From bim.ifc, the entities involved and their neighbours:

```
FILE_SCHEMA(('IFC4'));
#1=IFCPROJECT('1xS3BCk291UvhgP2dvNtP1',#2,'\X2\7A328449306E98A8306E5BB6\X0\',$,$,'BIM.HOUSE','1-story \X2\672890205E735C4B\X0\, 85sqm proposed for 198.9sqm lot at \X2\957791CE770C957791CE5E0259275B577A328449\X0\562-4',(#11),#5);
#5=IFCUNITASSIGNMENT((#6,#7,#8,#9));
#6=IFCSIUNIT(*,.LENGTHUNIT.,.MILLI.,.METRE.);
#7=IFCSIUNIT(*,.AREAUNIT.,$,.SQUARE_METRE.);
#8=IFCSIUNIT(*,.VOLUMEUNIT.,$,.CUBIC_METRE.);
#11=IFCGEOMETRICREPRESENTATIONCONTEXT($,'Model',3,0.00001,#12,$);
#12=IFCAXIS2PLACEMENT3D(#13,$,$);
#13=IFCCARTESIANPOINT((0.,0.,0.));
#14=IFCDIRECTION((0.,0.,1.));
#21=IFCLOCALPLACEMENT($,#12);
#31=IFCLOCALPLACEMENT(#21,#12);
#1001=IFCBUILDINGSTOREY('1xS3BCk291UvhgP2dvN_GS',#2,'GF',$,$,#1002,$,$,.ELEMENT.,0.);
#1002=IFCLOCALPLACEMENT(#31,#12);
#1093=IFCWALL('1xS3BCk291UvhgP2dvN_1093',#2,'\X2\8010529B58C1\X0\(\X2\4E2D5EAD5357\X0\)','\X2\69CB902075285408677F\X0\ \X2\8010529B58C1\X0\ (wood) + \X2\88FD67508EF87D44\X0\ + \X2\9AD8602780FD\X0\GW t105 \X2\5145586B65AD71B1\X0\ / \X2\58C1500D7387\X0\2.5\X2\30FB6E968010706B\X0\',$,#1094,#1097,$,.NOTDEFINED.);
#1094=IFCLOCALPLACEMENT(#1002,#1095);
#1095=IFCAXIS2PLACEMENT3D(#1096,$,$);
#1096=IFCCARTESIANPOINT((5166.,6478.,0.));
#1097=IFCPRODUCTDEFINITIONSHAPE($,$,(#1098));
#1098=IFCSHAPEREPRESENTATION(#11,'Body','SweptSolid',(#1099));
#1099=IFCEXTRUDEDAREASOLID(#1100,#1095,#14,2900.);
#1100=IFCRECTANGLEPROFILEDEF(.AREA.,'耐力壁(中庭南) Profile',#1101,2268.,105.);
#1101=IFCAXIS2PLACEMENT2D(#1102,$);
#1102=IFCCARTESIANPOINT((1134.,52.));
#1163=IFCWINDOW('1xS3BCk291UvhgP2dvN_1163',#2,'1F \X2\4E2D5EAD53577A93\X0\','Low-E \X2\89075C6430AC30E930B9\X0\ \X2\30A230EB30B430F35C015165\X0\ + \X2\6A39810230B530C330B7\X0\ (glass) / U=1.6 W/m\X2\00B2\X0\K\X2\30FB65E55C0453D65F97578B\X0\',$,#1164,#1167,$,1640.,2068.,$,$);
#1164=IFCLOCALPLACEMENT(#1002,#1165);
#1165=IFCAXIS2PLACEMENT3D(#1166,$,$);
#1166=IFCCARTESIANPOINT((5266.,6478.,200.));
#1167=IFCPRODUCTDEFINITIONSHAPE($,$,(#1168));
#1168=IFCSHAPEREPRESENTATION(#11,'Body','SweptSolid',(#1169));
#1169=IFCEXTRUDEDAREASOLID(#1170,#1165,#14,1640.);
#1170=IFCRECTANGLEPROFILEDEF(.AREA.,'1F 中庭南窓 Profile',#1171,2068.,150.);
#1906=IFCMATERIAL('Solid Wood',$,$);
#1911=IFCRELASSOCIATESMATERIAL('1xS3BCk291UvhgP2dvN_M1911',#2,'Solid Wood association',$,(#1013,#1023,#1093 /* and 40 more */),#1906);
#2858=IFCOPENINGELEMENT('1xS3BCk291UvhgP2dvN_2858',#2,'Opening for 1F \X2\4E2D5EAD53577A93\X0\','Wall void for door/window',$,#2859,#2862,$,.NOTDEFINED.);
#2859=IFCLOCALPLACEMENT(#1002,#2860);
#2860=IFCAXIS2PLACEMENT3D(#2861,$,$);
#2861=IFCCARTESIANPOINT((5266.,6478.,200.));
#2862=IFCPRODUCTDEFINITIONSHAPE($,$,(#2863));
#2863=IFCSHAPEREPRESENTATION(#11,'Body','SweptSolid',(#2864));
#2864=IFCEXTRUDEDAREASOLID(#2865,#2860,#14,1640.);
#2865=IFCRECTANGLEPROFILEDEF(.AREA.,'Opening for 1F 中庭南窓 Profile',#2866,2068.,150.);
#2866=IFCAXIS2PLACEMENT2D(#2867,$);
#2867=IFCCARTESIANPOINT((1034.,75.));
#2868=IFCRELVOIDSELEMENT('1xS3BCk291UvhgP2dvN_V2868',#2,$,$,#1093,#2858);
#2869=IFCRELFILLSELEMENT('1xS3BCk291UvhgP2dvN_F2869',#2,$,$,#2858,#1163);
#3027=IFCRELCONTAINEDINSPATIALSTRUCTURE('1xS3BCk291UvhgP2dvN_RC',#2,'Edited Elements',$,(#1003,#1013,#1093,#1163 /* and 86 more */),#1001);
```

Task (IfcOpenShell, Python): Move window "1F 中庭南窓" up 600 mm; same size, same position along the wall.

```python
import numpy as np
import ifcopenshell
import ifcopenshell.api.geometry
import ifcopenshell.util.placement
import ifcopenshell.util.unit

model = ifcopenshell.open("bim.ifc")
unit_scale = ifcopenshell.util.unit.calculate_unit_scale(model)

window = model.by_guid("1xS3BCk291UvhgP2dvN_1163")
opening = window.FillsVoids[0].RelatingOpeningElement
dz = 600.0

shift = np.array([0.0, 0.0, dz])
# The window is not placed relative to its opening, so move both.
for product in (opening, window):
    matrix = ifcopenshell.util.placement.get_local_placement(product.ObjectPlacement)
    matrix[:3, 3] += shift
    ifcopenshell.api.geometry.edit_object_placement(model, product=product, matrix=matrix, is_si=False)

print(f"moved by {dz * unit_scale:+.3f} m")

model.write("bim_edited.ifc")
```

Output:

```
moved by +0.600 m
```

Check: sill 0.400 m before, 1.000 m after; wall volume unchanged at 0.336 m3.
